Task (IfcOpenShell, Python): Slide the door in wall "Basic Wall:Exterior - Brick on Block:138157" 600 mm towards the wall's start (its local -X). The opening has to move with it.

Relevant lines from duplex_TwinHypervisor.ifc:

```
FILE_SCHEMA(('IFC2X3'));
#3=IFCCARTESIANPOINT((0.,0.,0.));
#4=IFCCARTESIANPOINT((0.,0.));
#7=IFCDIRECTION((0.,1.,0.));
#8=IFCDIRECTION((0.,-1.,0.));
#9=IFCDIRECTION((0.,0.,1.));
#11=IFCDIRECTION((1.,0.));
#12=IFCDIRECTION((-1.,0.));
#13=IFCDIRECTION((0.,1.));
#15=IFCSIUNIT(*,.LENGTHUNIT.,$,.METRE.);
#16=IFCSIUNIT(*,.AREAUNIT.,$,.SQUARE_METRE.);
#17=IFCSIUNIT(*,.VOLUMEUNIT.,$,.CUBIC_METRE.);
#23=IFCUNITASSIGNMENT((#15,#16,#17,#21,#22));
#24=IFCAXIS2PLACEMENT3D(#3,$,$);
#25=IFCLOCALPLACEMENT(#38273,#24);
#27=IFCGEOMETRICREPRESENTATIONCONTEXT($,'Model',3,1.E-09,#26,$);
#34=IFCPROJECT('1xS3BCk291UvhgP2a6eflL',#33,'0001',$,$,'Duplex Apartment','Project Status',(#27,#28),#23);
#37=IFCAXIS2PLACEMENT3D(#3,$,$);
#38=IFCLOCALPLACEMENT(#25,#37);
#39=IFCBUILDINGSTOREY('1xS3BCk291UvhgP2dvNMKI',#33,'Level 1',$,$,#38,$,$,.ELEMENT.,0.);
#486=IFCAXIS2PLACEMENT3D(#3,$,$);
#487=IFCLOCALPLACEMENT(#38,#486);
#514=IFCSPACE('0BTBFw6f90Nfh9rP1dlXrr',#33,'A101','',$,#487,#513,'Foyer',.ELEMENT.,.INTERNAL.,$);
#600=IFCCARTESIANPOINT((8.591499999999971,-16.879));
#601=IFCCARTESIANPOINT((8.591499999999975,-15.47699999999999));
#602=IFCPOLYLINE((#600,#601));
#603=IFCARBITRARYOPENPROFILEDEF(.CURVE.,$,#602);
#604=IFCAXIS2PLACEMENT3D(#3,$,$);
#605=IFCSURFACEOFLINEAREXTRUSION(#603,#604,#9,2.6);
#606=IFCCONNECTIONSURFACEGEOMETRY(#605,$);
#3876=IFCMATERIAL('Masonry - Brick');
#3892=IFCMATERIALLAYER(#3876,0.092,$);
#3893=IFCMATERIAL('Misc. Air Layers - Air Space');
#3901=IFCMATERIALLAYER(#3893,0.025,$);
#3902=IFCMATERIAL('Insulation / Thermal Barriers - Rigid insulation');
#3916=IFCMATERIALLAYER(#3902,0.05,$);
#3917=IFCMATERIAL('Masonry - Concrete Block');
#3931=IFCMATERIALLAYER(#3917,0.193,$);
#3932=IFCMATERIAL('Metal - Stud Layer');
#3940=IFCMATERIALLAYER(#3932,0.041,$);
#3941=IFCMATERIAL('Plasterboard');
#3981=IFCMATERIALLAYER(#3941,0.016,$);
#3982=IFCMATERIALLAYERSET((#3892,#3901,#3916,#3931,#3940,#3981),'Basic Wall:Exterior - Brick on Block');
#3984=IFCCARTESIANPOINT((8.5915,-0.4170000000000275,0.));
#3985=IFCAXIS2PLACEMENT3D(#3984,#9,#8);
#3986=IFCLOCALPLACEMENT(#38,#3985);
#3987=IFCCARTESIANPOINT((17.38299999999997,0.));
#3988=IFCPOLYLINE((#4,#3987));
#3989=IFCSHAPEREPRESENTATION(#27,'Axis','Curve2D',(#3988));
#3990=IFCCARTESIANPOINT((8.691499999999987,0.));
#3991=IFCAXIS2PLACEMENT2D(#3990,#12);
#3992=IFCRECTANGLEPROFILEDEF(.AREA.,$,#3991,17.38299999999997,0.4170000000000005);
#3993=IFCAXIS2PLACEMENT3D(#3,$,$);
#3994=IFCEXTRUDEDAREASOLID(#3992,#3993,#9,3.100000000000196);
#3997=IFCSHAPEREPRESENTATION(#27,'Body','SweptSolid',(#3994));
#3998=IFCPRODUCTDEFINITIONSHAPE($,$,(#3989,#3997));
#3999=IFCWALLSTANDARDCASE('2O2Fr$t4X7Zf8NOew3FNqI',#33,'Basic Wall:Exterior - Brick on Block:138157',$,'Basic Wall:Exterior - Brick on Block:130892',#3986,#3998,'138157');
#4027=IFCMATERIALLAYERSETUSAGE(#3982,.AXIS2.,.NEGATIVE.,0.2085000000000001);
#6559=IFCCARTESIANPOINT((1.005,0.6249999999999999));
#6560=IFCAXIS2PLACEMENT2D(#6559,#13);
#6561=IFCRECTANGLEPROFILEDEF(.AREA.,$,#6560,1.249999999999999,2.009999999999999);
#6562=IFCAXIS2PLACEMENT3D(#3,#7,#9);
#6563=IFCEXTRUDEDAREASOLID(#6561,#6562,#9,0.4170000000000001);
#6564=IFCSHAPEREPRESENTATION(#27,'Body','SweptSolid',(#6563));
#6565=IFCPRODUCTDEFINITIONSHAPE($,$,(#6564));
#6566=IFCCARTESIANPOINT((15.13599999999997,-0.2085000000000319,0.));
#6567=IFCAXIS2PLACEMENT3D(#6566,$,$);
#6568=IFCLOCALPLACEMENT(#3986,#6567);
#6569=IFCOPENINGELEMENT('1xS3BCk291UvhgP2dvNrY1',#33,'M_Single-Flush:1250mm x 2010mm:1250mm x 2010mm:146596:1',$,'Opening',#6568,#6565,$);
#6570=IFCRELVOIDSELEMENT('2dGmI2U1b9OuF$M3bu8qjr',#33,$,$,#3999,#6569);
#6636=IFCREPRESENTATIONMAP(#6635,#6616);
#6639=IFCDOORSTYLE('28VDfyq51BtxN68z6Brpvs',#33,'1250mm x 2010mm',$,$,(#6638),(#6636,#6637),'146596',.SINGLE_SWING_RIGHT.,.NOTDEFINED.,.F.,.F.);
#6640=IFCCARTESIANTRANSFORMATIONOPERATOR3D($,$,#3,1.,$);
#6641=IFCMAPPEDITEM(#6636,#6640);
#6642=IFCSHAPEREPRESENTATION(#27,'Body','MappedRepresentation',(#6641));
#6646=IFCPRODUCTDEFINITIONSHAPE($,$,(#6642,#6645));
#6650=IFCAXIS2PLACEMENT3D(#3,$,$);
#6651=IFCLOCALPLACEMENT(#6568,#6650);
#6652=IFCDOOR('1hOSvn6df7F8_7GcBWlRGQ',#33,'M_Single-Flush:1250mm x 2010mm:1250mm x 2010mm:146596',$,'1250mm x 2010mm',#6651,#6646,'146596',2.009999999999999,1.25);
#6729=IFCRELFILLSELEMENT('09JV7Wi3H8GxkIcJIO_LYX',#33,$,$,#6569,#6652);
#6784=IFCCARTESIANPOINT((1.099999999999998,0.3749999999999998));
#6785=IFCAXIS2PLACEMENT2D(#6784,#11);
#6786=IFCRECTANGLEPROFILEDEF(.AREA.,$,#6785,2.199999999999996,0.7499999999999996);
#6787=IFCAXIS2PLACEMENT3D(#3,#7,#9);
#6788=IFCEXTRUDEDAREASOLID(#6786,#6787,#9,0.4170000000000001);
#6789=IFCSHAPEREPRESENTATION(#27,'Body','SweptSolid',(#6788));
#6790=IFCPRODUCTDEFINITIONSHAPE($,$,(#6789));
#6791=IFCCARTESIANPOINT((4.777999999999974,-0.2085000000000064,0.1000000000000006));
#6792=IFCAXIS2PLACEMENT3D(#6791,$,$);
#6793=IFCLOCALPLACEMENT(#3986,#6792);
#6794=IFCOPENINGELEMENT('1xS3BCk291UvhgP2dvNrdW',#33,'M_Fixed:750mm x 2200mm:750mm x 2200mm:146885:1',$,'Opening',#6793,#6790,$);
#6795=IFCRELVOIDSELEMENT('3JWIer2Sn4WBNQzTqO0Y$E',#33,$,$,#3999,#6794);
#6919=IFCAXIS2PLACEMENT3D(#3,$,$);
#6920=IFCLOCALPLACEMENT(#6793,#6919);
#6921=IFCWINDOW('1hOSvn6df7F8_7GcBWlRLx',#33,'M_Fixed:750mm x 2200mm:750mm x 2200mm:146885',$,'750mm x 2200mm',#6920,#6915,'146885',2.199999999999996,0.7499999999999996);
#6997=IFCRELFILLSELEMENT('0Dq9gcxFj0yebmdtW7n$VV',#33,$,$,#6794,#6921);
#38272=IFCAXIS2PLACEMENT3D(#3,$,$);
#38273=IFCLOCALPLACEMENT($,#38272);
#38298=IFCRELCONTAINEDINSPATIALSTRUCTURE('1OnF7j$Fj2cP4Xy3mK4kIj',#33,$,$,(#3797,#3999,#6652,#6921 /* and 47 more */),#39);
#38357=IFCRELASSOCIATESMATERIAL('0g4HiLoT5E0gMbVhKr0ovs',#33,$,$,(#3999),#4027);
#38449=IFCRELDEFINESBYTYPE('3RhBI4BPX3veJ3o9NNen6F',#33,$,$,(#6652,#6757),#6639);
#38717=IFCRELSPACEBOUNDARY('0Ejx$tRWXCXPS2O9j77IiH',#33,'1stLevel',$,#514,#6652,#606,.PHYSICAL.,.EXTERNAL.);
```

```python
import numpy as np
import ifcopenshell
import ifcopenshell.api.geometry
import ifcopenshell.util.placement

model = ifcopenshell.open("duplex_TwinHypervisor.ifc")

door = model.by_guid("1hOSvn6df7F8_7GcBWlRGQ")
opening = door.FillsVoids[0].RelatingOpeningElement
wall = opening.VoidsElements[0].RelatingBuildingElement

wall_matrix = ifcopenshell.util.placement.get_local_placement(wall.ObjectPlacement)
shift = wall_matrix[:3, 0] * -0.6
before = ifcopenshell.util.placement.get_local_placement(door.ObjectPlacement)[:3, 3].copy()

# The door is placed relative to its opening, so it follows when the opening moves.
matrix = ifcopenshell.util.placement.get_local_placement(opening.ObjectPlacement)
matrix[:3, 3] += shift
ifcopenshell.api.geometry.edit_object_placement(
    model, product=opening, matrix=matrix, is_si=False, should_transform_children=True
)

# Space boundary surfaces are stored in each space's coordinates; move them too.
for rel in door.ProvidesBoundaries:
    if not rel.ConnectionGeometry:
        continue
    surface = rel.ConnectionGeometry.SurfaceOnRelatingElement
    space_matrix = ifcopenshell.util.placement.get_local_placement(rel.RelatingSpace.ObjectPlacement)
    point = np.array(surface.Position.Location.Coordinates) + space_matrix[:3, :3].T @ shift
    surface.Position = model.createIfcAxis2Placement3D(
        model.createIfcCartesianPoint(point.tolist()), surface.Position.Axis, surface.Position.RefDirection
    )

after = ifcopenshell.util.placement.get_local_placement(door.ObjectPlacement)[:3, 3]
print("door moved by", (after - before).round(3) + 0.0)

model.write("duplex_TwinHypervisor-out.ifc")
```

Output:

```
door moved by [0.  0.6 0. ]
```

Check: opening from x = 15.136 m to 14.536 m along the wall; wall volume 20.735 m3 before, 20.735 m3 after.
